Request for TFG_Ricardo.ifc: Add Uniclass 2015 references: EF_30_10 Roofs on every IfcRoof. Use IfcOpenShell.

First a look at what the model holds.

```python
import ifcopenshell

model = ifcopenshell.open("TFG_Ricardo.ifc")
print(model.schema)
print("classifications:", [c.Name for c in model.by_type("IfcClassification")])
for ifc_class in ("IfcDoor", "IfcRoof", "IfcStair", "IfcWall", "IfcWindow"):
    print(ifc_class, len(model.by_type(ifc_class)))
```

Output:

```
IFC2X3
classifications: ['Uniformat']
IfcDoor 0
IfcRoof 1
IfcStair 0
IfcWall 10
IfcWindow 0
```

```python
import ifcopenshell
import ifcopenshell.api.classification

model = ifcopenshell.open("TFG_Ricardo.ifc")

# IFC2X3 requires Source and Edition and has no link from the project to the system.
system = model.create_entity("IfcClassification", Source="NBS", Edition="2015", Name="Uniclass 2015")

codes = {
    "IfcRoof": ("EF_30_10", "Roofs"),
}
for ifc_class, (code, name) in codes.items():
    products = model.by_type(ifc_class)
    ifcopenshell.api.classification.add_reference(
        model, products=products, classification=system, identification=code, name=name
    )
    print(code, len(products))

model.write("TFG_Ricardo_updated.ifc")
```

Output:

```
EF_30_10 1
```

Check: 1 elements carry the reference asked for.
